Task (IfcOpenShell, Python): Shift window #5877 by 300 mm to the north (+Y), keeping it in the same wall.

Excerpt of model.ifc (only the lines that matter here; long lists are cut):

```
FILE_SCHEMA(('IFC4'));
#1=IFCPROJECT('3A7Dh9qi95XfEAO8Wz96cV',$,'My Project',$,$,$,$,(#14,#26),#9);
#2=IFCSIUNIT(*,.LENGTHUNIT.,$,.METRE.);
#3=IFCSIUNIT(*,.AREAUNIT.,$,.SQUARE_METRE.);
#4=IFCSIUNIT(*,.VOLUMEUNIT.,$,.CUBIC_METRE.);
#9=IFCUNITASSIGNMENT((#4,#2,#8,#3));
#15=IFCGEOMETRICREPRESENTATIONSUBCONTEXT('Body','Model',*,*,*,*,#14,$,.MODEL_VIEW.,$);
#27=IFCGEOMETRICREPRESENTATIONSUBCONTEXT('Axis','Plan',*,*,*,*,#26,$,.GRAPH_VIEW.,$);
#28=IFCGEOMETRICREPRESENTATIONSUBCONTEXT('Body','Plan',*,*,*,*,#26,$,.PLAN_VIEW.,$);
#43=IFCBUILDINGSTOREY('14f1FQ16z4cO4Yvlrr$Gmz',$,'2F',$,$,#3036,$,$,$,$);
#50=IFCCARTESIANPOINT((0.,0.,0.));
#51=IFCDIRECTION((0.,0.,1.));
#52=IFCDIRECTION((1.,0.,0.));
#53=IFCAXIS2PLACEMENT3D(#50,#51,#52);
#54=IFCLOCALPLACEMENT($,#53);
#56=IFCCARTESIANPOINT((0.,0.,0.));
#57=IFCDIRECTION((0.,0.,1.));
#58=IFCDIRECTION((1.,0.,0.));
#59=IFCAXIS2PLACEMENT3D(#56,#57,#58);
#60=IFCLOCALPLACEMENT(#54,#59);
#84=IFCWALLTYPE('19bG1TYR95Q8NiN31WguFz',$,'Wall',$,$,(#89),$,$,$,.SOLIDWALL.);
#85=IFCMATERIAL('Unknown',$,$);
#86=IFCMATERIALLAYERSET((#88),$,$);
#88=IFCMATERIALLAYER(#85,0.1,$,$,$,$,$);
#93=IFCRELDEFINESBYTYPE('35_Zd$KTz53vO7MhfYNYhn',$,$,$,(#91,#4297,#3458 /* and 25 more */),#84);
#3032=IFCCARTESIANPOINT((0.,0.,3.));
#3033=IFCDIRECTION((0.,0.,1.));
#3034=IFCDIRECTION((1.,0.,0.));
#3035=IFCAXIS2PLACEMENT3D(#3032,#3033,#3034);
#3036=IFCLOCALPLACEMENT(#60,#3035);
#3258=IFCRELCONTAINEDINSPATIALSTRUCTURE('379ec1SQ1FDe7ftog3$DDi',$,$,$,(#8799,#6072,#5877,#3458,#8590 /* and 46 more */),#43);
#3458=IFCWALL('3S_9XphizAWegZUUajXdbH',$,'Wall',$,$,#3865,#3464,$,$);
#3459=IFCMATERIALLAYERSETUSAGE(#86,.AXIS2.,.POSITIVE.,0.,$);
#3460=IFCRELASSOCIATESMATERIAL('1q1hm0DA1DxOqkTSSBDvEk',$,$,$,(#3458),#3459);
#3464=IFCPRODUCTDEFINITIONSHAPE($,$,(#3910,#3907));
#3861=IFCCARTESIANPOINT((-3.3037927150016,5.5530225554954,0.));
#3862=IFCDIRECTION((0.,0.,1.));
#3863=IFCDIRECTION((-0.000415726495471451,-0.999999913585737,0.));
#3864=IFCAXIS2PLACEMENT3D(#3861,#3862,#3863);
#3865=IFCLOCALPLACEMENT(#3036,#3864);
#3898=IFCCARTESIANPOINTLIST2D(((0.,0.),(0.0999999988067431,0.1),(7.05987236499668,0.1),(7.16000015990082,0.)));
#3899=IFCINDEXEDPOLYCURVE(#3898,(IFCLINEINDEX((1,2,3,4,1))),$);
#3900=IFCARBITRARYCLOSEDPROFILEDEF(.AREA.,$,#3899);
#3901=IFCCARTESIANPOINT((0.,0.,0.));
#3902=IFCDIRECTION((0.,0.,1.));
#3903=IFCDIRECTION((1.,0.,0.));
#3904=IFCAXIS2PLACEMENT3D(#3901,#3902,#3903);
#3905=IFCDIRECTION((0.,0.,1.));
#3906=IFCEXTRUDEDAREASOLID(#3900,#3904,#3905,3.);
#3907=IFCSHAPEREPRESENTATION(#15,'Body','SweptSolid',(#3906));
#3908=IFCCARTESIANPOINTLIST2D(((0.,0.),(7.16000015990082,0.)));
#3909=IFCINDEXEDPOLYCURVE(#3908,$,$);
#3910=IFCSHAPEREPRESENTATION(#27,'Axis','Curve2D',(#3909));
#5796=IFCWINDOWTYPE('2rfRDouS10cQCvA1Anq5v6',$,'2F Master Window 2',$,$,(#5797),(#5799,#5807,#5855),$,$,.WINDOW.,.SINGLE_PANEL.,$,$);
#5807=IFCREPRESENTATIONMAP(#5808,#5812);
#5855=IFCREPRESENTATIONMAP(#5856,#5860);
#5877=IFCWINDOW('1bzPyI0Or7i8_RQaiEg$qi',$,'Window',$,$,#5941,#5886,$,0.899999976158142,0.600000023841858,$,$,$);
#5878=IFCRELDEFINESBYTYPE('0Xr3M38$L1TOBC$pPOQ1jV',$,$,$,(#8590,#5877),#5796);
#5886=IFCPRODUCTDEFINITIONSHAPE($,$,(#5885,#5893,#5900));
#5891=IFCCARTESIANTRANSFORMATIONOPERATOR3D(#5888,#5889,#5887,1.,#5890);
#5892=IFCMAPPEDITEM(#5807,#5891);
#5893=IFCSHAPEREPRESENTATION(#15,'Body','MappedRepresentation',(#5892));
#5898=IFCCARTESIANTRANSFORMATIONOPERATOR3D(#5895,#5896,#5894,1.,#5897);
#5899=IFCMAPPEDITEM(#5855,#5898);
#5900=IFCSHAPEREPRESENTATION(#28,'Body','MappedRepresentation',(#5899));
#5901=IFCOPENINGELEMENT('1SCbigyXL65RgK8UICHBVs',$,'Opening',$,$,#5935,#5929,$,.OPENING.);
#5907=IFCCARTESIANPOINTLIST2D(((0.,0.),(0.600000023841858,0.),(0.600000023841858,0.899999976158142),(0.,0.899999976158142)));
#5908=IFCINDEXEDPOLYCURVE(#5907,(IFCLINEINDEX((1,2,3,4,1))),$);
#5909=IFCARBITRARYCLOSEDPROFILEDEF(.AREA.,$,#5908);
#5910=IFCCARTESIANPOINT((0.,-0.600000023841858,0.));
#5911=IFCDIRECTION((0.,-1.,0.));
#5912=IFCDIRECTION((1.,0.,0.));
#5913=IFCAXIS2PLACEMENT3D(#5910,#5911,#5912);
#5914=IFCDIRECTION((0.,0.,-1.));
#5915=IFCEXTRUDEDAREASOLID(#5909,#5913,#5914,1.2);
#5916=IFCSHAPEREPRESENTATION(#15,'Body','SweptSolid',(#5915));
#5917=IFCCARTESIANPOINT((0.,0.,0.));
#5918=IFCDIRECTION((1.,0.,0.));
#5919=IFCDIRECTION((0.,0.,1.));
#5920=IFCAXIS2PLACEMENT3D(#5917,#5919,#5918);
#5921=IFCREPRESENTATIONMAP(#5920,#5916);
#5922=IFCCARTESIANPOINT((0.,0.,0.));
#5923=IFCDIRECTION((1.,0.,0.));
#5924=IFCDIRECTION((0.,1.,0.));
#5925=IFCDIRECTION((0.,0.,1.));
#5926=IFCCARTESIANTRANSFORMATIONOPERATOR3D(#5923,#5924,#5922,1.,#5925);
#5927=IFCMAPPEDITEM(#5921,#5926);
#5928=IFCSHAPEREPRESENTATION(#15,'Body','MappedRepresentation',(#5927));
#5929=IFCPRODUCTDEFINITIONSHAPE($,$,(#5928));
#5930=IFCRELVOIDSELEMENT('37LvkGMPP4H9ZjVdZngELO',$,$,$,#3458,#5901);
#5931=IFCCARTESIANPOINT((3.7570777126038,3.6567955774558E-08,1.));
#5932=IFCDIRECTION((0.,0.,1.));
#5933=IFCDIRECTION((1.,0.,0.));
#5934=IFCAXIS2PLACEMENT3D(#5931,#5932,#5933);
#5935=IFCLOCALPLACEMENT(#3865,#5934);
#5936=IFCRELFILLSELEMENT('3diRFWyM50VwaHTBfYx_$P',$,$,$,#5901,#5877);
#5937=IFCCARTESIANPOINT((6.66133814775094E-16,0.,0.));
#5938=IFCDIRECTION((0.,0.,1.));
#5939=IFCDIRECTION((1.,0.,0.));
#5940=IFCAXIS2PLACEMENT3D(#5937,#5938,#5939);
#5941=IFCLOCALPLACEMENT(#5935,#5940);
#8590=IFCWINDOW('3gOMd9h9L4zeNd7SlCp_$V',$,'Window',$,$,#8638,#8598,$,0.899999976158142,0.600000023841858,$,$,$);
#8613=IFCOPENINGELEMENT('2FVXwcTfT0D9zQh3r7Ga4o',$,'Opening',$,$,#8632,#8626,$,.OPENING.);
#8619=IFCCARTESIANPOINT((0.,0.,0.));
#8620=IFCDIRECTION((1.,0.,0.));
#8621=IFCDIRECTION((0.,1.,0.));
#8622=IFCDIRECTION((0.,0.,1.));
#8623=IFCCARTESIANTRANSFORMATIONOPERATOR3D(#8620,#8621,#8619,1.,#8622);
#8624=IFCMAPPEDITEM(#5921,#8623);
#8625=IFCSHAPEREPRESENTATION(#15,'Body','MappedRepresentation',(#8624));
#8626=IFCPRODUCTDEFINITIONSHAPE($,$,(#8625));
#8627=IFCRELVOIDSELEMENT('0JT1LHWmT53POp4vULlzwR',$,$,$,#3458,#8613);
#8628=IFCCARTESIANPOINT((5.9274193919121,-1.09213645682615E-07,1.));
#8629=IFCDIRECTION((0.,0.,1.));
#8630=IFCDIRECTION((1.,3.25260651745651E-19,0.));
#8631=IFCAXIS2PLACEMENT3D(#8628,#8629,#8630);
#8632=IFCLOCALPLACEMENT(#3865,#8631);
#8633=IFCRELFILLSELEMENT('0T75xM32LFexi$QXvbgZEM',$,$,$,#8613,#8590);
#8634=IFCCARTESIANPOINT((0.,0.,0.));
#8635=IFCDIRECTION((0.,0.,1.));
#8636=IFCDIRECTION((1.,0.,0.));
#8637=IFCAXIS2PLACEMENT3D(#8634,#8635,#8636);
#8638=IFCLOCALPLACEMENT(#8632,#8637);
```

```python
import ifcopenshell
import ifcopenshell.api.geometry
import ifcopenshell.util.placement

model = ifcopenshell.open("model.ifc")

window = model.by_guid("1bzPyI0Or7i8_RQaiEg$qi")
opening = window.FillsVoids[0].RelatingOpeningElement
wall = opening.VoidsElements[0].RelatingBuildingElement

wall_matrix = ifcopenshell.util.placement.get_local_placement(wall.ObjectPlacement)
shift = wall_matrix[:3, 0] * -0.3
before = ifcopenshell.util.placement.get_local_placement(window.ObjectPlacement)[:3, 3].copy()

# The window is placed relative to its opening, so it follows when the opening moves.
matrix = ifcopenshell.util.placement.get_local_placement(opening.ObjectPlacement)
matrix[:3, 3] += shift
ifcopenshell.api.geometry.edit_object_placement(
    model, product=opening, matrix=matrix, is_si=False, should_transform_children=True
)

after = ifcopenshell.util.placement.get_local_placement(window.ObjectPlacement)[:3, 3]
print("window moved by", (after - before).round(3) + 0.0)

model.write("model-out.ifc")
```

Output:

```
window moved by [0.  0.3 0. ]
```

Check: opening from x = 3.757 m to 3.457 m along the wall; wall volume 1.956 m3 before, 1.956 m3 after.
